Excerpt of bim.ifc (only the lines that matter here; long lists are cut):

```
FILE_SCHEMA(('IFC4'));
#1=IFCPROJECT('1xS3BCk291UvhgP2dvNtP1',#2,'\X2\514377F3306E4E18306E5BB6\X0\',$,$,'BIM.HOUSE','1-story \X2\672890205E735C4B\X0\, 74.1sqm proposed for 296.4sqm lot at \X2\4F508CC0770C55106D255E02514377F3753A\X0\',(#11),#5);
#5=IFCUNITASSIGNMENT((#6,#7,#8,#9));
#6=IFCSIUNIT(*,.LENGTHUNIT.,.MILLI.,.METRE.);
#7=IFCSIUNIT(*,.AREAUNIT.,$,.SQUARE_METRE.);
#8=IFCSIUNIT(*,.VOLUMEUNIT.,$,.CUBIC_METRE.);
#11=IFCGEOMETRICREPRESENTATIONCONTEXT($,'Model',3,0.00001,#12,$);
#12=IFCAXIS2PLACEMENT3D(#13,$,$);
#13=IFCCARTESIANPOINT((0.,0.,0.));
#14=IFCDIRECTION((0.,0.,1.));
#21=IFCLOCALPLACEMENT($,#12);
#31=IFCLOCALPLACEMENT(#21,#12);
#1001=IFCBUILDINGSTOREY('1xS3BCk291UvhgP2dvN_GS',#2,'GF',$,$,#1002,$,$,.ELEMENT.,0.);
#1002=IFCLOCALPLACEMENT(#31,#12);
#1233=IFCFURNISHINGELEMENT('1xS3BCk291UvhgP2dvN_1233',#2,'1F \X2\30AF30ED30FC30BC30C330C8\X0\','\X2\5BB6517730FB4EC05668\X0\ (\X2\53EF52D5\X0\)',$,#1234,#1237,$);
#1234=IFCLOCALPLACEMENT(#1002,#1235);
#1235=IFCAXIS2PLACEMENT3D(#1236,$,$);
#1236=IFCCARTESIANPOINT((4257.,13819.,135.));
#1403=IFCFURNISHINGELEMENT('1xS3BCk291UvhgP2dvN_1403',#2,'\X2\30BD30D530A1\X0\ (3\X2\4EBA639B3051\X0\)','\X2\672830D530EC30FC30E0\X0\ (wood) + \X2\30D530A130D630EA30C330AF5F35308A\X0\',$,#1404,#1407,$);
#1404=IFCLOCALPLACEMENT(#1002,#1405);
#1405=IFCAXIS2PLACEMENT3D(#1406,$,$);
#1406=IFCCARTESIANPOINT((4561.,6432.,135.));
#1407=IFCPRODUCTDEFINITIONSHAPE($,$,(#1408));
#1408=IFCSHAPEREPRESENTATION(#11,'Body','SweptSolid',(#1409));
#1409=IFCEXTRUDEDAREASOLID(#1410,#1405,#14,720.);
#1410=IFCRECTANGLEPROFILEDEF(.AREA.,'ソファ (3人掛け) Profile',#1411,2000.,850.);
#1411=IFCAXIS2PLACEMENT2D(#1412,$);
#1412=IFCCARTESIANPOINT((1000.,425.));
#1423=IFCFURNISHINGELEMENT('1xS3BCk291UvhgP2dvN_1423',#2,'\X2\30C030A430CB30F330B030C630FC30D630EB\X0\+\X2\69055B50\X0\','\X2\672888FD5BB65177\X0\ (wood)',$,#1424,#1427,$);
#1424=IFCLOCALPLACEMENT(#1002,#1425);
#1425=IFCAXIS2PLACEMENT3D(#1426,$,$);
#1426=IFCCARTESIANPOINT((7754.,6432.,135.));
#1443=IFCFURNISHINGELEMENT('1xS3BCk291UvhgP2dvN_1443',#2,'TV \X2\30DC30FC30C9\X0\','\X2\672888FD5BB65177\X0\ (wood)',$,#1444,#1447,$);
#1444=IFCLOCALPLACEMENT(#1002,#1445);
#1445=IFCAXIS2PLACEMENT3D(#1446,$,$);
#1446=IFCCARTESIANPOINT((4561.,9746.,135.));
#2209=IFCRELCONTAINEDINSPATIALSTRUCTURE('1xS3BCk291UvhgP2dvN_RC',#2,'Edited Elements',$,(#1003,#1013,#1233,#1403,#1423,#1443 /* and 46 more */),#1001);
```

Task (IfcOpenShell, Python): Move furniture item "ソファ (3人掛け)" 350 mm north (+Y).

```python
import ifcopenshell
import ifcopenshell.api.geometry
import ifcopenshell.util.placement

model = ifcopenshell.open("bim.ifc")

item = model.by_id(1403)
matrix = ifcopenshell.util.placement.get_local_placement(item.ObjectPlacement)
matrix[1, 3] += 350.0
ifcopenshell.api.geometry.edit_object_placement(model, product=item, matrix=matrix, is_si=False)

print(ifcopenshell.util.placement.get_local_placement(item.ObjectPlacement).round(3) + 0.0)

model.write("bim-out.ifc")
```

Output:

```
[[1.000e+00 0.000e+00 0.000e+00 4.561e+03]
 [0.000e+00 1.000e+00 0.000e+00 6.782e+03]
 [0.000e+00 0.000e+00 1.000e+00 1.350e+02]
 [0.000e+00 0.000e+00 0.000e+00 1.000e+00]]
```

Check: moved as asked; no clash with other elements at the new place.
